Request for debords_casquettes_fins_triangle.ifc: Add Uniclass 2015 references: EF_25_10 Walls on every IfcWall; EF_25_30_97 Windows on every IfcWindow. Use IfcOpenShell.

First a look at what the model holds.

```python
import ifcopenshell

model = ifcopenshell.open("debords_casquettes_fins_triangle.ifc")
print(model.schema)
print("classifications:", [c.Name for c in model.by_type("IfcClassification")])
for ifc_class in ("IfcDoor", "IfcRoof", "IfcStair", "IfcWall", "IfcWindow"):
    print(ifc_class, len(model.by_type(ifc_class)))
```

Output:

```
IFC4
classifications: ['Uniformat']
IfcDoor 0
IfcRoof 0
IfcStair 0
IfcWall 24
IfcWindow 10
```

```python
import ifcopenshell
import ifcopenshell.api.classification

model = ifcopenshell.open("debords_casquettes_fins_triangle.ifc")

system = ifcopenshell.api.classification.add_classification(model, classification="Uniclass 2015")

codes = {
    "IfcWall": ("EF_25_10", "Walls"),
    "IfcWindow": ("EF_25_30_97", "Windows"),
}
for ifc_class, (code, name) in codes.items():
    products = model.by_type(ifc_class)
    ifcopenshell.api.classification.add_reference(
        model, products=products, classification=system, identification=code, name=name
    )
    print(code, len(products))

model.write("debords_casquettes_fins_triangle_edited.ifc")
```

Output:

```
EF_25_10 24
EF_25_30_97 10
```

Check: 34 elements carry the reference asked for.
